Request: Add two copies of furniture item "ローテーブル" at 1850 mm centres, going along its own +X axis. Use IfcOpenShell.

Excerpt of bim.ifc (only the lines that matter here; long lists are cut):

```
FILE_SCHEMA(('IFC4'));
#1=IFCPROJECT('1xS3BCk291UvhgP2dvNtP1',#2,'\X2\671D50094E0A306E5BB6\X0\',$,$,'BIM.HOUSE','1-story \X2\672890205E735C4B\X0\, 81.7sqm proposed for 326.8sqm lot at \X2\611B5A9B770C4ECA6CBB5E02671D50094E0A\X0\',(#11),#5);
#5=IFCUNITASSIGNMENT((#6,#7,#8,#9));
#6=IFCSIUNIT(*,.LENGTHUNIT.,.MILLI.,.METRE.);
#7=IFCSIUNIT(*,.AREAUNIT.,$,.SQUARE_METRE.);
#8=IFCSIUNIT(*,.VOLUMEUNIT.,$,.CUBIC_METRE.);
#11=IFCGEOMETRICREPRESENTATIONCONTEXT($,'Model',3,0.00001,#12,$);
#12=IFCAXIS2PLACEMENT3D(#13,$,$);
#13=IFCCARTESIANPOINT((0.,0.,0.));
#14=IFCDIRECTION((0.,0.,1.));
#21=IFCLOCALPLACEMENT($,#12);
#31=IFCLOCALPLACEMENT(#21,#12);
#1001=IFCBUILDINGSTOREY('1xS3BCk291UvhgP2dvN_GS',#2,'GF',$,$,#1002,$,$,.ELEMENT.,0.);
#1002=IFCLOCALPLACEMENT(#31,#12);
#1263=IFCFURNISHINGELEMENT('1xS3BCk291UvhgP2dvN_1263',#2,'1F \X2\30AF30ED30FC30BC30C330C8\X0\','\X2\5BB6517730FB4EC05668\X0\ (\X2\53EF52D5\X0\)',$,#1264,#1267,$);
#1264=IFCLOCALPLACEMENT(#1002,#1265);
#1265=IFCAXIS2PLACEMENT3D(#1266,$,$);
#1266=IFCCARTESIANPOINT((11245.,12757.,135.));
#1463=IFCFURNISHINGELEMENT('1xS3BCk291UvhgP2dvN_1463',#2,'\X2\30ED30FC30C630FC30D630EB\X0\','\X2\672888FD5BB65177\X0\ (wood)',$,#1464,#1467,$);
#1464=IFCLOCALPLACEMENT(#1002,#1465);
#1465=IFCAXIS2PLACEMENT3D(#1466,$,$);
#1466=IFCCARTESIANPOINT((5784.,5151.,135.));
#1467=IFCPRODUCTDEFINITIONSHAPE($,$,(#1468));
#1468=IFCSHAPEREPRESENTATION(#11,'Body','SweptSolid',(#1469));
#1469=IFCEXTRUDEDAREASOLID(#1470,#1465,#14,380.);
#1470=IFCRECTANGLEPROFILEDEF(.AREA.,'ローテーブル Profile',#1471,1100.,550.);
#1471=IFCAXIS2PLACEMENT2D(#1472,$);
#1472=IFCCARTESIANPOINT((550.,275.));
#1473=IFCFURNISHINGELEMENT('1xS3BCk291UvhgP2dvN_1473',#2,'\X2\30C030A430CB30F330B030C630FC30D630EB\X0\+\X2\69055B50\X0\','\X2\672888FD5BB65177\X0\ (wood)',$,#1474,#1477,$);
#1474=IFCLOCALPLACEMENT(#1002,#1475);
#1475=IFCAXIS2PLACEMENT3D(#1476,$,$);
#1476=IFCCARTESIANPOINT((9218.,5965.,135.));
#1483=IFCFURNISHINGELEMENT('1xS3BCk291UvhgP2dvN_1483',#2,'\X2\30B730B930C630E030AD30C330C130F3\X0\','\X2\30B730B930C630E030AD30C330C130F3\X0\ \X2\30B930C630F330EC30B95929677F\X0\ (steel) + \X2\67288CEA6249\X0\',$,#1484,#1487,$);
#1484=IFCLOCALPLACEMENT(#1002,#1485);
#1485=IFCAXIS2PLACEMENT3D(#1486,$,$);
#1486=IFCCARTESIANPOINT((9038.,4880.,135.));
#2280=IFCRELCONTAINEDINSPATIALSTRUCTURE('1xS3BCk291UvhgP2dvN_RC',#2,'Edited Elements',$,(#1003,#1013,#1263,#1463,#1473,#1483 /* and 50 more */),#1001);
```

```python
import ifcopenshell
import ifcopenshell.api.geometry
import ifcopenshell.api.root
import ifcopenshell.util.element
import ifcopenshell.util.placement

model = ifcopenshell.open("bim.ifc")


def reuse_history(source, copy):
    """copy_class also copies each property set's owner history, people and application; keep the originals."""
    for rel in copy.IsDefinedBy:
        if rel.is_a("IfcRelDefinesByProperties") and (history := rel.RelatingPropertyDefinition.OwnerHistory):
            rel.RelatingPropertyDefinition.OwnerHistory = source.OwnerHistory
            ifcopenshell.util.element.remove_deep2(model, history)


source = model.by_guid("1xS3BCk291UvhgP2dvN_1463")
base = ifcopenshell.util.placement.get_local_placement(source.ObjectPlacement)
step = base[:3, 0] * 1850.0

for i in range(1, 3):
    copy = ifcopenshell.api.root.copy_class(model, product=source)
    copy.Representation = ifcopenshell.util.element.copy_deep(
        model, source.Representation, exclude=["IfcGeometricRepresentationContext", "IfcRepresentationMap"]
    )
    reuse_history(source, copy)
    matrix = base.copy()
    matrix[:3, 3] += i * step
    print("added at", matrix[:3, 3].round(3) + 0.0)
    ifcopenshell.api.geometry.edit_object_placement(model, product=copy, matrix=matrix, is_si=False)

model.write("bim_v2.ifc")
```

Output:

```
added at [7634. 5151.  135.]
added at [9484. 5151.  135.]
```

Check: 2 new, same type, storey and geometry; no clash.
